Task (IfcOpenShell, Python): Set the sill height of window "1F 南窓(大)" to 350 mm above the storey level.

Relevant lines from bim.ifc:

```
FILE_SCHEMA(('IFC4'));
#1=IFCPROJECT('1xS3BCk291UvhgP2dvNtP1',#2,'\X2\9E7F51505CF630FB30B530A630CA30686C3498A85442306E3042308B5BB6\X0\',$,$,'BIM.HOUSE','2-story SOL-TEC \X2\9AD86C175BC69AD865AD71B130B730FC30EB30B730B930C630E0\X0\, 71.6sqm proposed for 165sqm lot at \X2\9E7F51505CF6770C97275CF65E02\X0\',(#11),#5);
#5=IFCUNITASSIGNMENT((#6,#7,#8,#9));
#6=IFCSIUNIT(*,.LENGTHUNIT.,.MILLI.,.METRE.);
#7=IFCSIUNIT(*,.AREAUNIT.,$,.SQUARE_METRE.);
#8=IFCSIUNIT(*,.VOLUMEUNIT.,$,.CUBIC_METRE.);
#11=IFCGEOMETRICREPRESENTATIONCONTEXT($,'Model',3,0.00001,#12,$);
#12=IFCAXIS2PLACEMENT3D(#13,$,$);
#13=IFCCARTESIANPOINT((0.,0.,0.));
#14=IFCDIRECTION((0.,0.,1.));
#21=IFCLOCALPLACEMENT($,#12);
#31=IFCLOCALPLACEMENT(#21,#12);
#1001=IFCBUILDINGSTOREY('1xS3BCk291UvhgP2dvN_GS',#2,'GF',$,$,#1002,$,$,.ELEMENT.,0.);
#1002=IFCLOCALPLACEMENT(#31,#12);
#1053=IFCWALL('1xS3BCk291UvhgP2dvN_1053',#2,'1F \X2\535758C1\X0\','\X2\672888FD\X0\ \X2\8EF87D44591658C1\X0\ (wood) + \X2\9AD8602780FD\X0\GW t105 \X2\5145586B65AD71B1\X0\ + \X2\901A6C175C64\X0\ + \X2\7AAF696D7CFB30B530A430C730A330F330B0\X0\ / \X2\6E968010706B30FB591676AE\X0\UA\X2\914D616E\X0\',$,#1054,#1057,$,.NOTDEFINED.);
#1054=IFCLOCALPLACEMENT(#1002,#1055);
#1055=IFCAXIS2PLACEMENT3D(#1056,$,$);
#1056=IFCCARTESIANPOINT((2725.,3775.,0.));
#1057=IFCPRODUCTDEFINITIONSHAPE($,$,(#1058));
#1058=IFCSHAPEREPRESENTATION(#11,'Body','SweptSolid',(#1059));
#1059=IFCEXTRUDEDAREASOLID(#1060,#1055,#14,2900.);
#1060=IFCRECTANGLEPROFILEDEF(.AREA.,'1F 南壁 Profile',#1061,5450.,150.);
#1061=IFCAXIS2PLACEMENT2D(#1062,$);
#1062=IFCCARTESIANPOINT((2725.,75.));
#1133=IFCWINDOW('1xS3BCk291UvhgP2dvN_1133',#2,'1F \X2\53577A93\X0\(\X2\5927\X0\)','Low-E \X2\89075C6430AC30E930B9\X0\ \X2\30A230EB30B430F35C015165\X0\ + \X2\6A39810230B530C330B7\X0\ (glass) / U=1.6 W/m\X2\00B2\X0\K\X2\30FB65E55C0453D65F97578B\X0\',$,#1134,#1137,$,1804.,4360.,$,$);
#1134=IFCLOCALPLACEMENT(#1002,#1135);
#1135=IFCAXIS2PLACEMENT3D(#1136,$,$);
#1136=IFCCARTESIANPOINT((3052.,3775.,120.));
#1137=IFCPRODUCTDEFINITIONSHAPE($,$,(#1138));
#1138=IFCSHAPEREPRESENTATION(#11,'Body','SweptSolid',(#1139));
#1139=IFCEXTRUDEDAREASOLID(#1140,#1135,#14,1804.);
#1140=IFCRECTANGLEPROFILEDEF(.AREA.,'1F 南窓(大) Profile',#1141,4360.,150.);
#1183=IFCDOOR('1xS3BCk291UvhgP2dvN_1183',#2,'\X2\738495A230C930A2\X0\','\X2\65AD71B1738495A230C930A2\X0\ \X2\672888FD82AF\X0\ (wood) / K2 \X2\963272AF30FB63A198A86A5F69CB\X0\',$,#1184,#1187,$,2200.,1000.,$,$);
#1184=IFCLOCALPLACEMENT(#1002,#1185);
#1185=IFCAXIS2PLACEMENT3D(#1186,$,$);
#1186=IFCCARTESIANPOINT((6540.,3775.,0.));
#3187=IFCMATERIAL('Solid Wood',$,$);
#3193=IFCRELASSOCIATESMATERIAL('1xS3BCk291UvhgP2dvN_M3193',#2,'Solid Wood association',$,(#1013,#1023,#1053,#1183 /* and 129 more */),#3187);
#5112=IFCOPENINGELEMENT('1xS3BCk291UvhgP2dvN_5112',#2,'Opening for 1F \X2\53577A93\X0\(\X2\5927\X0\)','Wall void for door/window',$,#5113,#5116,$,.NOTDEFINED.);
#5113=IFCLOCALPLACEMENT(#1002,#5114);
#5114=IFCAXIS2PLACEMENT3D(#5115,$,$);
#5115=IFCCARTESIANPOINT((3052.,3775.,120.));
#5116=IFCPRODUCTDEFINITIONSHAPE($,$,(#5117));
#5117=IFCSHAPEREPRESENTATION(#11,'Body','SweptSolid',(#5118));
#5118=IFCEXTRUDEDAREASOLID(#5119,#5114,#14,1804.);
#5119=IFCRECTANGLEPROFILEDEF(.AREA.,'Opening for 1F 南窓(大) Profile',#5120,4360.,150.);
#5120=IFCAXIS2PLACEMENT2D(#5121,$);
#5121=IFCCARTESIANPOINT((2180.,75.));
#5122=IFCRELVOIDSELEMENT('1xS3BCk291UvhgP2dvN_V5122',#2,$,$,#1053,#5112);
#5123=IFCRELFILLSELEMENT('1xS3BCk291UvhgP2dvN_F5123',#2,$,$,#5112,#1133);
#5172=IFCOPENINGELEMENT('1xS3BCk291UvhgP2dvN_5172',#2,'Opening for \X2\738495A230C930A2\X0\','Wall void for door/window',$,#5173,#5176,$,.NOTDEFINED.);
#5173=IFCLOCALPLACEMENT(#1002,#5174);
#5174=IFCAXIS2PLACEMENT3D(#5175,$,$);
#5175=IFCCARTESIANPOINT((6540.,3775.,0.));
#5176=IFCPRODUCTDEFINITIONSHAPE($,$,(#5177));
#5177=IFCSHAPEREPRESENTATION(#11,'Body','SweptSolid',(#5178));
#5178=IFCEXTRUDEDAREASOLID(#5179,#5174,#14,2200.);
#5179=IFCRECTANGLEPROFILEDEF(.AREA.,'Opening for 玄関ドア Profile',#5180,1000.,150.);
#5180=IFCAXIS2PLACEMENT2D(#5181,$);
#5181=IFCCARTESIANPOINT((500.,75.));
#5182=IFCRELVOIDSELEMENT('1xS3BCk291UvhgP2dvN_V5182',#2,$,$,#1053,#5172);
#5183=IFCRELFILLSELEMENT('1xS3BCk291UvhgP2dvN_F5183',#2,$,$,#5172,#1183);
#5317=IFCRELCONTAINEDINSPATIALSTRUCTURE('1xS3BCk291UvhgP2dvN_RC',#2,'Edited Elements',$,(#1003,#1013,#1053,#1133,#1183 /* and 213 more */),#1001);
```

```python
import numpy as np
import ifcopenshell
import ifcopenshell.api.geometry
import ifcopenshell.geom
import ifcopenshell.util.element
import ifcopenshell.util.placement
import ifcopenshell.util.shape
import ifcopenshell.util.unit

model = ifcopenshell.open("bim.ifc")
unit_scale = ifcopenshell.util.unit.calculate_unit_scale(model)

window = model.by_guid("1xS3BCk291UvhgP2dvN_1133")
opening = window.FillsVoids[0].RelatingOpeningElement
storey = ifcopenshell.util.element.get_container(window, ifc_class="IfcBuildingStorey")
level = ifcopenshell.util.placement.get_local_placement(storey.ObjectPlacement)[2, 3]

# The opening's origin need not be at the sill, so measure its lowest point.
shape = ifcopenshell.geom.create_shape(ifcopenshell.geom.settings(), opening)
bottom = ifcopenshell.util.shape.get_shape_bottom_elevation(shape, shape.geometry) / unit_scale
dz = level + 0.35 / unit_scale - bottom

shift = np.array([0.0, 0.0, dz])
# The window is not placed relative to its opening, so move both.
for product in (opening, window):
    matrix = ifcopenshell.util.placement.get_local_placement(product.ObjectPlacement)
    matrix[:3, 3] += shift
    ifcopenshell.api.geometry.edit_object_placement(model, product=product, matrix=matrix, is_si=False)

print(f"moved by {dz * unit_scale:+.3f} m")

model.write("bim_edited.ifc")
```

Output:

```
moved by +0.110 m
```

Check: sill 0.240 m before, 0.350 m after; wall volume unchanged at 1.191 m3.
